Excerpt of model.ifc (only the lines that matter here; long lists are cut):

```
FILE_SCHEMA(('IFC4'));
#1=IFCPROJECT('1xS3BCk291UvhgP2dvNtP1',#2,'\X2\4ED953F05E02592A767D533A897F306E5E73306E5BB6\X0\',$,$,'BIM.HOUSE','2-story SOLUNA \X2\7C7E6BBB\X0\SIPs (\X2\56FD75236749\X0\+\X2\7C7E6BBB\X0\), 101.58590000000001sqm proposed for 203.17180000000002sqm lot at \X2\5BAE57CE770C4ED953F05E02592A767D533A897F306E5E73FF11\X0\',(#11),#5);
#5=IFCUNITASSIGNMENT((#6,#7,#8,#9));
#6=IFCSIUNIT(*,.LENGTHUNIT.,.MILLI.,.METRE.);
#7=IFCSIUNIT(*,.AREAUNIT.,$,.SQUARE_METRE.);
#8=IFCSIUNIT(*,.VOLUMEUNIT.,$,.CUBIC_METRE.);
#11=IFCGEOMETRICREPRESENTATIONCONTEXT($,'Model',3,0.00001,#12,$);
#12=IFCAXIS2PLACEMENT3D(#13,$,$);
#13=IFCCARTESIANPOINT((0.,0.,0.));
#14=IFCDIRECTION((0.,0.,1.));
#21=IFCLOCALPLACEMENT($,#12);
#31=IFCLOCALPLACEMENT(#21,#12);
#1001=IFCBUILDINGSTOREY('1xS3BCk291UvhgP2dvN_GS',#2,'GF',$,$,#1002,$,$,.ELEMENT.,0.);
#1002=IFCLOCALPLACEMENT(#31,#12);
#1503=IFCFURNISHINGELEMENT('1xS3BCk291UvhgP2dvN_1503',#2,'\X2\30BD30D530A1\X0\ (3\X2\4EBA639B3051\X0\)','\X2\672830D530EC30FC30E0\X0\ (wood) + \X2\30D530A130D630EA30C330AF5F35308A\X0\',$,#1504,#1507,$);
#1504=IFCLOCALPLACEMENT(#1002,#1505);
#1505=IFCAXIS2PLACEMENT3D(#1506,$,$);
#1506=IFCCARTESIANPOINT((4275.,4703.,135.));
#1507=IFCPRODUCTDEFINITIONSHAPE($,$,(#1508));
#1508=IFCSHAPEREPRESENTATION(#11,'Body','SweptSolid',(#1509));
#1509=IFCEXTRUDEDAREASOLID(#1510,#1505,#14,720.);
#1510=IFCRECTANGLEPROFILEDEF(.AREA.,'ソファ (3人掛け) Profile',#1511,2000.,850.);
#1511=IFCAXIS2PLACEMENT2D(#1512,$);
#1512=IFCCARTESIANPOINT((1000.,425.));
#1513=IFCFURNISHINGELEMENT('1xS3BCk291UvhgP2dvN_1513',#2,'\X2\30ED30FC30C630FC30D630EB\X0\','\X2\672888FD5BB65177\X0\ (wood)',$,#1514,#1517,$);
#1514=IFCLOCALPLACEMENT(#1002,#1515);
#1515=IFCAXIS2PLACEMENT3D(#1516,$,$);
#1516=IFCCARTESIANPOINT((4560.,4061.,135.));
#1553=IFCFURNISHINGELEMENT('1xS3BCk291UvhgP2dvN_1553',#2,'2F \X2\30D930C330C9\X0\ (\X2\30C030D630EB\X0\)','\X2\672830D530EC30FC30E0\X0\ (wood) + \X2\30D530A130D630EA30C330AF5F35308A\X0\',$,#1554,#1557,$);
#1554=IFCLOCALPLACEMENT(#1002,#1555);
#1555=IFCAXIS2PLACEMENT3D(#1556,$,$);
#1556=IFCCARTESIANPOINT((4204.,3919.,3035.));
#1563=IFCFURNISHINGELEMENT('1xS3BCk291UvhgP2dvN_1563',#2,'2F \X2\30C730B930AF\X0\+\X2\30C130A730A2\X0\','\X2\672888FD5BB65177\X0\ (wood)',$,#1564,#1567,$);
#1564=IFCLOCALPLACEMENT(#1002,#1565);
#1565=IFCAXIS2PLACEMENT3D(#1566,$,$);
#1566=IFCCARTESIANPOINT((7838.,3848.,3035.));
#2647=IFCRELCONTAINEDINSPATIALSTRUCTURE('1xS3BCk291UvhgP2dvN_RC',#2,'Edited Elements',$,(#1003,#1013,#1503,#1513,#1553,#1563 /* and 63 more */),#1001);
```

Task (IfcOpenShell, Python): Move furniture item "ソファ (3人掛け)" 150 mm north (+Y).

```python
import ifcopenshell
import ifcopenshell.api.geometry
import ifcopenshell.util.placement

model = ifcopenshell.open("model.ifc")

item = model.by_guid("1xS3BCk291UvhgP2dvN_1503")
matrix = ifcopenshell.util.placement.get_local_placement(item.ObjectPlacement)
matrix[1, 3] += 150.0
ifcopenshell.api.geometry.edit_object_placement(model, product=item, matrix=matrix, is_si=False)

print(ifcopenshell.util.placement.get_local_placement(item.ObjectPlacement).round(3) + 0.0)

model.write("model_rev.ifc")
```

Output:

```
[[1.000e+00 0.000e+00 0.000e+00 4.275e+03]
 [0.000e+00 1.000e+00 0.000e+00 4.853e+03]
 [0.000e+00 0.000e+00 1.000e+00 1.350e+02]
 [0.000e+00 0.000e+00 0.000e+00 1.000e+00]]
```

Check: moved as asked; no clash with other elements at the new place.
